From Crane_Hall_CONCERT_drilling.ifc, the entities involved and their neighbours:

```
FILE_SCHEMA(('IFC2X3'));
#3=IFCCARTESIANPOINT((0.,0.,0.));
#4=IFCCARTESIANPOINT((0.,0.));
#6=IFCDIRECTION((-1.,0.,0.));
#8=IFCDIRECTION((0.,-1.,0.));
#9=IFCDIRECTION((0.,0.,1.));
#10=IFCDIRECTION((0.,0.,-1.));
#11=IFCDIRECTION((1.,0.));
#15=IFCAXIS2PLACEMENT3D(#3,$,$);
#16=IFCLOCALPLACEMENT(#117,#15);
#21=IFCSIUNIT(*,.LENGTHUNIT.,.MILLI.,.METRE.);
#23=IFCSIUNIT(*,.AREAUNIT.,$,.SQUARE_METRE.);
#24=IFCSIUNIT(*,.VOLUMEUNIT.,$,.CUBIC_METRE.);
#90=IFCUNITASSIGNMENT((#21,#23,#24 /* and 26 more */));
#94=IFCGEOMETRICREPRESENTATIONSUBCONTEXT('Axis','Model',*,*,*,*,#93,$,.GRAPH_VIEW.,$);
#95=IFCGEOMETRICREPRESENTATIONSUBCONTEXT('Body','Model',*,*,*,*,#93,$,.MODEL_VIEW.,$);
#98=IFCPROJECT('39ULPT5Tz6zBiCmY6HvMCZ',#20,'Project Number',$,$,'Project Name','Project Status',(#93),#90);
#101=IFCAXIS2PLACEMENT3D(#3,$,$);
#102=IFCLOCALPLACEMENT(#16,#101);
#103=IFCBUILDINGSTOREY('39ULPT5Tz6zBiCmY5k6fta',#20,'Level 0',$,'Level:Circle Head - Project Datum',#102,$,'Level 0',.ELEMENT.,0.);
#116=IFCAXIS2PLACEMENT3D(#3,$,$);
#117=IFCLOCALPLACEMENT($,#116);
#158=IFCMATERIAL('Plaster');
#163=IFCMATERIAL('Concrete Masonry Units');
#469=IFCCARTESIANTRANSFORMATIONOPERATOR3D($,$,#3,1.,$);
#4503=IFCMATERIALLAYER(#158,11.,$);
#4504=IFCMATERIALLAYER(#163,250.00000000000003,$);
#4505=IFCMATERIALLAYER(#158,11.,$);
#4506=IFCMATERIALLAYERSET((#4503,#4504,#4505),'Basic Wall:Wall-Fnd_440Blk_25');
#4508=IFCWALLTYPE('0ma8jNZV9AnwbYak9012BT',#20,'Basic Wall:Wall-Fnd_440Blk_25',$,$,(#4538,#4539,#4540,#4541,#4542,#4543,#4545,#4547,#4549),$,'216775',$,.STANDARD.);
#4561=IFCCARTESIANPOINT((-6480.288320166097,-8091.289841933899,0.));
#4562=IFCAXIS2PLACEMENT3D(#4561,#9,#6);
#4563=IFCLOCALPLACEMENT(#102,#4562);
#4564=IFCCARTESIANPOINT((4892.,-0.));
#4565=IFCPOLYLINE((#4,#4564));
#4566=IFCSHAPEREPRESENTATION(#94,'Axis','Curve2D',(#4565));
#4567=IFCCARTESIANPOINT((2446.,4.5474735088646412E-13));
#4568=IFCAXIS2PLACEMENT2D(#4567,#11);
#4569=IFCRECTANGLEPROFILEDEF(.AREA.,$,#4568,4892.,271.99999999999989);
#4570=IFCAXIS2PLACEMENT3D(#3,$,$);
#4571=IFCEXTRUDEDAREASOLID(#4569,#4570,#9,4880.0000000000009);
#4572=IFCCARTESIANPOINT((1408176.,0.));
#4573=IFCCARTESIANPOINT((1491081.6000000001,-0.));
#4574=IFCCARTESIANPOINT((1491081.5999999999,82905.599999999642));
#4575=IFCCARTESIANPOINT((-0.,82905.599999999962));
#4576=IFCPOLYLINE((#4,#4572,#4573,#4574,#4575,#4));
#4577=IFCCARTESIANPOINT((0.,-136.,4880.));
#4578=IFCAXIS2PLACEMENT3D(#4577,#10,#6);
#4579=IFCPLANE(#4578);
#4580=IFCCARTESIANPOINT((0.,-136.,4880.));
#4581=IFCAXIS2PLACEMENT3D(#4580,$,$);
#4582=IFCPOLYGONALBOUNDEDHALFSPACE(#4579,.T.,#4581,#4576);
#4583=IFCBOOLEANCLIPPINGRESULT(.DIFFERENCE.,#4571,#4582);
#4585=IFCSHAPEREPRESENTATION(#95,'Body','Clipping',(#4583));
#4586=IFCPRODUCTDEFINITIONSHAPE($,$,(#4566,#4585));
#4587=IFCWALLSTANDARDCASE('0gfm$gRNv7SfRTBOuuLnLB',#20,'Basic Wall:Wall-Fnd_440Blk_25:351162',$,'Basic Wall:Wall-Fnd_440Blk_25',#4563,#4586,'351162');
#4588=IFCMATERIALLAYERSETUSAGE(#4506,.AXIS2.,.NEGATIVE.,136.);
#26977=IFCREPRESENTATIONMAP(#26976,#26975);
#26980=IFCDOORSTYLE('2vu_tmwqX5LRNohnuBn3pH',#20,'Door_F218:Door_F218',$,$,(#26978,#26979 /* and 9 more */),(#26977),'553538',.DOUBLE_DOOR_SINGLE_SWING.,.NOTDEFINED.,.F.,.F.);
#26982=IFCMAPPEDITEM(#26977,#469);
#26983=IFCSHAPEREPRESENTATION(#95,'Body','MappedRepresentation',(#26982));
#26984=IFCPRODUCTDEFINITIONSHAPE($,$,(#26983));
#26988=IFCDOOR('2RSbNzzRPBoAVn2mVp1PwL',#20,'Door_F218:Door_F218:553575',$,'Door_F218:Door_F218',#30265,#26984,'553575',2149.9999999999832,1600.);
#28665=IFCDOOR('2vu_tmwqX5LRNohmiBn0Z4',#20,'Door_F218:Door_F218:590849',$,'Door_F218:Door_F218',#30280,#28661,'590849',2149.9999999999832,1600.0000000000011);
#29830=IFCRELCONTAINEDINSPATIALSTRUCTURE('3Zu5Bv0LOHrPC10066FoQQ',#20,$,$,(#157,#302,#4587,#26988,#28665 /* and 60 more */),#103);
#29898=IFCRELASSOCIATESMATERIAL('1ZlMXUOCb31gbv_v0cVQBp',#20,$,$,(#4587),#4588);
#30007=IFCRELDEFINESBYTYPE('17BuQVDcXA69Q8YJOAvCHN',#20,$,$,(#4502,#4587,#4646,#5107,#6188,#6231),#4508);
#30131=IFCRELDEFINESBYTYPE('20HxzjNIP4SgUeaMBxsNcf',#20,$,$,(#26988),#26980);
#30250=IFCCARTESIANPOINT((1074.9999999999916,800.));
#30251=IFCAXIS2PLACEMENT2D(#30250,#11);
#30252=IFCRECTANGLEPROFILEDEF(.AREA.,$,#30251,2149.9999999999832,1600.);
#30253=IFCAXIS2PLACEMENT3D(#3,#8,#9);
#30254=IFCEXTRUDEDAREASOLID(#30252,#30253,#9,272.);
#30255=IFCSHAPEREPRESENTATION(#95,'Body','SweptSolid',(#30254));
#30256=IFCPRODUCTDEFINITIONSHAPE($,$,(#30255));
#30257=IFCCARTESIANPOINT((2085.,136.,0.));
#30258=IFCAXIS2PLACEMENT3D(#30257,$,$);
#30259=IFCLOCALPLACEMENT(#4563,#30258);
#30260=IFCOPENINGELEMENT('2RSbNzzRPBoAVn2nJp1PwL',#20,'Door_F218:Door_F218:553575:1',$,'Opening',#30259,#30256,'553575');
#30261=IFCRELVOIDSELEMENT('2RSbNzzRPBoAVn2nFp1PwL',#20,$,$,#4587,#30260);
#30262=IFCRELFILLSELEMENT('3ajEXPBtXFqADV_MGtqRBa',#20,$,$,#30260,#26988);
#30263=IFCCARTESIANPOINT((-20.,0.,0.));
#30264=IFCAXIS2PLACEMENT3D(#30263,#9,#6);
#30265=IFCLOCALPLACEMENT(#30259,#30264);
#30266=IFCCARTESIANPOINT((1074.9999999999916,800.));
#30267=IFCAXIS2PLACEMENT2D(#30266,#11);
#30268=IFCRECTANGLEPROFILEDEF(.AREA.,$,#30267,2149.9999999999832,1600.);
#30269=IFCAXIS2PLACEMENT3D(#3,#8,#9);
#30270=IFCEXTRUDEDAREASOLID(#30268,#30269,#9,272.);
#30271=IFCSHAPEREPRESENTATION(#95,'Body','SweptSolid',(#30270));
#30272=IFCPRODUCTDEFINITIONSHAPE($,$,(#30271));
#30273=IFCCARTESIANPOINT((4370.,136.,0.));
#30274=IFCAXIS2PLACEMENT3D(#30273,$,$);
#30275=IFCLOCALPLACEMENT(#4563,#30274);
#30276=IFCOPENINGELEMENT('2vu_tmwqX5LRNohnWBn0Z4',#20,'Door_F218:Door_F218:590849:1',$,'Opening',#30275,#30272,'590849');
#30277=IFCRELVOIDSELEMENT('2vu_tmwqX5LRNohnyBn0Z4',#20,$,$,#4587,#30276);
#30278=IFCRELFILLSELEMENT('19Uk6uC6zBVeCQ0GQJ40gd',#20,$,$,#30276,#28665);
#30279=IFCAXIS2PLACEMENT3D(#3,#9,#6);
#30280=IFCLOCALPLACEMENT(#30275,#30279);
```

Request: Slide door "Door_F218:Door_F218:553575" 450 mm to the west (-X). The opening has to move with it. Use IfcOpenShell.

```python
import ifcopenshell
import ifcopenshell.api.geometry
import ifcopenshell.util.placement
import ifcopenshell.util.unit

model = ifcopenshell.open("Crane_Hall_CONCERT_drilling.ifc")
unit_scale = ifcopenshell.util.unit.calculate_unit_scale(model)

door = model.by_guid("2RSbNzzRPBoAVn2mVp1PwL")
opening = door.FillsVoids[0].RelatingOpeningElement
wall = opening.VoidsElements[0].RelatingBuildingElement

wall_matrix = ifcopenshell.util.placement.get_local_placement(wall.ObjectPlacement)
shift = wall_matrix[:3, 0] * 0.45 / unit_scale
before = ifcopenshell.util.placement.get_local_placement(door.ObjectPlacement)[:3, 3].copy()

# The door is placed relative to its opening, so it follows when the opening moves.
matrix = ifcopenshell.util.placement.get_local_placement(opening.ObjectPlacement)
matrix[:3, 3] += shift
ifcopenshell.api.geometry.edit_object_placement(
    model, product=opening, matrix=matrix, is_si=False, should_transform_children=True
)

after = ifcopenshell.util.placement.get_local_placement(door.ObjectPlacement)[:3, 3]
print("door moved by", (after - before).round(3) + 0.0)

model.write("Crane_Hall_CONCERT_drilling-out.ifc")
```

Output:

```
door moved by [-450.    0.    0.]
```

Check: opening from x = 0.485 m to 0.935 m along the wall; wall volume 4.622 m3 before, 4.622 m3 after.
